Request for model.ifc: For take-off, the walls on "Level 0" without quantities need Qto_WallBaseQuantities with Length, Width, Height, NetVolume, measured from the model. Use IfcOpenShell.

First a look at what the model holds.

```python
import ifcopenshell
import ifcopenshell.util.element
import ifcopenshell.util.unit

model = ifcopenshell.open("model.ifc")
print(model.schema)
for unit_type in ("LENGTHUNIT", "AREAUNIT", "VOLUMEUNIT"):
    print(unit_type, ifcopenshell.util.unit.calculate_unit_scale(model, unit_type))
storey = next(s for s in model.by_type("IfcBuildingStorey") if s.Name == "Level 0")
walls = [e for e in ifcopenshell.util.element.get_decomposition(storey) if e.is_a("IfcWall")]
for e in sorted(walls, key=lambda e: e.id()):
    print(e.id(), e.is_a(), e.Name, list(ifcopenshell.util.element.get_psets(e, qtos_only=True)), sep=" | ")
```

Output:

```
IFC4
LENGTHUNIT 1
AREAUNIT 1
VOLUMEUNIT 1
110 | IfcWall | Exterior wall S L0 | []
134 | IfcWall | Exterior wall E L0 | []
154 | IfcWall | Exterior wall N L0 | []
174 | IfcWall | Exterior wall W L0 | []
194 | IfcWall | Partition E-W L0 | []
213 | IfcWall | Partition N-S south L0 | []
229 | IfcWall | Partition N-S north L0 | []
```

```python
import ifcopenshell
import ifcopenshell.api.pset
import ifcopenshell.geom
import ifcopenshell.util.element
import ifcopenshell.util.shape
import ifcopenshell.util.unit

model = ifcopenshell.open("model.ifc")
unit_scale = ifcopenshell.util.unit.calculate_unit_scale(model)
volume_scale = ifcopenshell.util.unit.calculate_unit_scale(model, "VOLUMEUNIT")
settings = ifcopenshell.geom.settings()

storey = next(s for s in model.by_type("IfcBuildingStorey") if s.Name == "Level 0")
walls = [e for e in ifcopenshell.util.element.get_decomposition(storey) if e.is_a("IfcWall")]

for e in sorted(walls, key=lambda e: e.id()):
    if ifcopenshell.util.element.get_psets(e, qtos_only=True, should_inherit=False):
        continue
    # Geometry comes back in metres, in the element's own axes.
    shape = ifcopenshell.geom.create_shape(settings, e)
    values = {
        "Length": ifcopenshell.util.shape.get_x(shape.geometry) / unit_scale,
        "Width": ifcopenshell.util.shape.get_y(shape.geometry) / unit_scale,
        "Height": ifcopenshell.util.shape.get_z(shape.geometry) / unit_scale,
        "NetVolume": ifcopenshell.util.shape.get_volume(shape.geometry) / volume_scale,
    }
    qto = ifcopenshell.api.pset.add_qto(model, product=e, name="Qto_WallBaseQuantities")
    ifcopenshell.api.pset.edit_qto(model, qto=qto, properties=values)
    print(e.id(), {k: round(v, 3) for k, v in values.items()})

model.write("model-out.ifc")
```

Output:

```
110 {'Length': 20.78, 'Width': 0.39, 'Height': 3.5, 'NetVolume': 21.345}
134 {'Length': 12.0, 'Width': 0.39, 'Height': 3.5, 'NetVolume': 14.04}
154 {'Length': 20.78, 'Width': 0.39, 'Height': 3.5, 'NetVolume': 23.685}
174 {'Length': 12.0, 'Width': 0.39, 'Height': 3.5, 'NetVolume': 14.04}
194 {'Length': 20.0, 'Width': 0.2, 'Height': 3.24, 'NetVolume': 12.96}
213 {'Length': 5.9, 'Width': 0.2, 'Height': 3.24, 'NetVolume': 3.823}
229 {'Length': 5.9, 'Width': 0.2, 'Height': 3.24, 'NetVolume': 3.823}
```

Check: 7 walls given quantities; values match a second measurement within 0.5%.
